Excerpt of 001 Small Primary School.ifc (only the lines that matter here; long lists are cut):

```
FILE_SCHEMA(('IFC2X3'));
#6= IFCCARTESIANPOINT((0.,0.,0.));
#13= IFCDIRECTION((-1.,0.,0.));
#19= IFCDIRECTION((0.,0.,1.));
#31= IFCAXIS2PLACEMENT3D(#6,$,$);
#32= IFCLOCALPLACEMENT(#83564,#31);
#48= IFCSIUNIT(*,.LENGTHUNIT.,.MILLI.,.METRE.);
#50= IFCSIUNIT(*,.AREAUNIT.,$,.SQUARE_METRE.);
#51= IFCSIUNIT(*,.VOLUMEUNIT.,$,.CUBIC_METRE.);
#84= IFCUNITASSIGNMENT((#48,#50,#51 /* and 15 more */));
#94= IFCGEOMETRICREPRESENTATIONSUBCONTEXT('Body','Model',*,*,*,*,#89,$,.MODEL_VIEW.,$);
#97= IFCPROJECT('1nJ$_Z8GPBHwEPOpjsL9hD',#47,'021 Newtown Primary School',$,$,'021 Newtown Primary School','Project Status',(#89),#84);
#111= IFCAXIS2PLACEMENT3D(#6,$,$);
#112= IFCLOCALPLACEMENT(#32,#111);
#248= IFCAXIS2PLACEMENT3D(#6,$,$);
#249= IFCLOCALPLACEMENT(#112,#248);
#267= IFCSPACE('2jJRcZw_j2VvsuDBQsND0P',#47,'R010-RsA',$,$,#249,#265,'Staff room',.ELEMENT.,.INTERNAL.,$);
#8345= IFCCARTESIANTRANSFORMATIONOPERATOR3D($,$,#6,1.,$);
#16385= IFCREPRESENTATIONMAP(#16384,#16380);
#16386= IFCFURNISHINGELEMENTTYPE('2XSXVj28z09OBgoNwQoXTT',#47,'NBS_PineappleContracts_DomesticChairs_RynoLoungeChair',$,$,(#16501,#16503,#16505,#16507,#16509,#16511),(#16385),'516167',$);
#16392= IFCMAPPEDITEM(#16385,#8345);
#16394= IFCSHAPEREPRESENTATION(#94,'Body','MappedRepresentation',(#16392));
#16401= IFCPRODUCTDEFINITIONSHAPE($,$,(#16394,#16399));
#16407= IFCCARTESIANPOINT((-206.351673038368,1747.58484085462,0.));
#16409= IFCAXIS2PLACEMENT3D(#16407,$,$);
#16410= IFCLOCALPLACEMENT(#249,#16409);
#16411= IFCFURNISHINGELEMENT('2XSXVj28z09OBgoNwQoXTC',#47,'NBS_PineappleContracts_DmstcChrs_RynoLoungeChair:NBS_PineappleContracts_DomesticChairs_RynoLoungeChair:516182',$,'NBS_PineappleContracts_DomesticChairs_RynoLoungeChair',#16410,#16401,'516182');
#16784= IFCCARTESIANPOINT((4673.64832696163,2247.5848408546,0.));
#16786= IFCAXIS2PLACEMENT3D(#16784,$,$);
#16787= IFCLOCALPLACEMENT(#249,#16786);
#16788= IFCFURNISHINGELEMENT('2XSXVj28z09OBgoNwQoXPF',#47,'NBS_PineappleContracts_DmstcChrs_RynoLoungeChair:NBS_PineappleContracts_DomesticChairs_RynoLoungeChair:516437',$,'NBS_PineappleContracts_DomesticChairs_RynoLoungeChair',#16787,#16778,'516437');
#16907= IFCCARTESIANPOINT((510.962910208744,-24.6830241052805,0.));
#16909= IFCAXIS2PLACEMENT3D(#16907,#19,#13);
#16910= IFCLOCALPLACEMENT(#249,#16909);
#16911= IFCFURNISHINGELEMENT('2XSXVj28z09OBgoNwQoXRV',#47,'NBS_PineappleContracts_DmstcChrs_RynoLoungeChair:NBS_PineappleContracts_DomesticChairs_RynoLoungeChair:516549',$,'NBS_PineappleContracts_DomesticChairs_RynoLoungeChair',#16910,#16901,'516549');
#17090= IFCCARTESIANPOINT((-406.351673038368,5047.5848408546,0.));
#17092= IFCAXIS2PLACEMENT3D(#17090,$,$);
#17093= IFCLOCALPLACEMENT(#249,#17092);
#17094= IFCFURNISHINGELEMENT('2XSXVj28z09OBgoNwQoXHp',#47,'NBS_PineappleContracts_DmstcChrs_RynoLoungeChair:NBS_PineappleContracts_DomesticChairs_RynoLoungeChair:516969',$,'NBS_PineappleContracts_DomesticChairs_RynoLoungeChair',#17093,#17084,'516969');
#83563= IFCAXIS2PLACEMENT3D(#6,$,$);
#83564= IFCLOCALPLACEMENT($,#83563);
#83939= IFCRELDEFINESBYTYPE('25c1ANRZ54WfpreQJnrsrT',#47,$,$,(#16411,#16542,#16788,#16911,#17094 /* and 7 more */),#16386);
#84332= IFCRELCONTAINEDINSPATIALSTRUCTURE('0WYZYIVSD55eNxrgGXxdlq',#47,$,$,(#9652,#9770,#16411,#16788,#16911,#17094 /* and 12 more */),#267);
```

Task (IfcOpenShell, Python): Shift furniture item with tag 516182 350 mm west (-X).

```python
import ifcopenshell
import ifcopenshell.api.geometry
import ifcopenshell.util.placement
import ifcopenshell.util.unit

model = ifcopenshell.open("001 Small Primary School.ifc")
unit_scale = ifcopenshell.util.unit.calculate_unit_scale(model)

item = model.by_guid("2XSXVj28z09OBgoNwQoXTC")
matrix = ifcopenshell.util.placement.get_local_placement(item.ObjectPlacement)
matrix[0, 3] -= 0.35 / unit_scale
ifcopenshell.api.geometry.edit_object_placement(model, product=item, matrix=matrix, is_si=False)

print(ifcopenshell.util.placement.get_local_placement(item.ObjectPlacement).round(3) + 0.0)

model.write("001 Small Primary School_v2.ifc")
```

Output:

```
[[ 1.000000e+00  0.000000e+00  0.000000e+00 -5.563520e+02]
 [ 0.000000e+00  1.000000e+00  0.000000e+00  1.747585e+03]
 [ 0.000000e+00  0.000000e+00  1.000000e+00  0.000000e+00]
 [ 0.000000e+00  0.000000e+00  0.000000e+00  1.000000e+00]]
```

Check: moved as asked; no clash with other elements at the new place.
